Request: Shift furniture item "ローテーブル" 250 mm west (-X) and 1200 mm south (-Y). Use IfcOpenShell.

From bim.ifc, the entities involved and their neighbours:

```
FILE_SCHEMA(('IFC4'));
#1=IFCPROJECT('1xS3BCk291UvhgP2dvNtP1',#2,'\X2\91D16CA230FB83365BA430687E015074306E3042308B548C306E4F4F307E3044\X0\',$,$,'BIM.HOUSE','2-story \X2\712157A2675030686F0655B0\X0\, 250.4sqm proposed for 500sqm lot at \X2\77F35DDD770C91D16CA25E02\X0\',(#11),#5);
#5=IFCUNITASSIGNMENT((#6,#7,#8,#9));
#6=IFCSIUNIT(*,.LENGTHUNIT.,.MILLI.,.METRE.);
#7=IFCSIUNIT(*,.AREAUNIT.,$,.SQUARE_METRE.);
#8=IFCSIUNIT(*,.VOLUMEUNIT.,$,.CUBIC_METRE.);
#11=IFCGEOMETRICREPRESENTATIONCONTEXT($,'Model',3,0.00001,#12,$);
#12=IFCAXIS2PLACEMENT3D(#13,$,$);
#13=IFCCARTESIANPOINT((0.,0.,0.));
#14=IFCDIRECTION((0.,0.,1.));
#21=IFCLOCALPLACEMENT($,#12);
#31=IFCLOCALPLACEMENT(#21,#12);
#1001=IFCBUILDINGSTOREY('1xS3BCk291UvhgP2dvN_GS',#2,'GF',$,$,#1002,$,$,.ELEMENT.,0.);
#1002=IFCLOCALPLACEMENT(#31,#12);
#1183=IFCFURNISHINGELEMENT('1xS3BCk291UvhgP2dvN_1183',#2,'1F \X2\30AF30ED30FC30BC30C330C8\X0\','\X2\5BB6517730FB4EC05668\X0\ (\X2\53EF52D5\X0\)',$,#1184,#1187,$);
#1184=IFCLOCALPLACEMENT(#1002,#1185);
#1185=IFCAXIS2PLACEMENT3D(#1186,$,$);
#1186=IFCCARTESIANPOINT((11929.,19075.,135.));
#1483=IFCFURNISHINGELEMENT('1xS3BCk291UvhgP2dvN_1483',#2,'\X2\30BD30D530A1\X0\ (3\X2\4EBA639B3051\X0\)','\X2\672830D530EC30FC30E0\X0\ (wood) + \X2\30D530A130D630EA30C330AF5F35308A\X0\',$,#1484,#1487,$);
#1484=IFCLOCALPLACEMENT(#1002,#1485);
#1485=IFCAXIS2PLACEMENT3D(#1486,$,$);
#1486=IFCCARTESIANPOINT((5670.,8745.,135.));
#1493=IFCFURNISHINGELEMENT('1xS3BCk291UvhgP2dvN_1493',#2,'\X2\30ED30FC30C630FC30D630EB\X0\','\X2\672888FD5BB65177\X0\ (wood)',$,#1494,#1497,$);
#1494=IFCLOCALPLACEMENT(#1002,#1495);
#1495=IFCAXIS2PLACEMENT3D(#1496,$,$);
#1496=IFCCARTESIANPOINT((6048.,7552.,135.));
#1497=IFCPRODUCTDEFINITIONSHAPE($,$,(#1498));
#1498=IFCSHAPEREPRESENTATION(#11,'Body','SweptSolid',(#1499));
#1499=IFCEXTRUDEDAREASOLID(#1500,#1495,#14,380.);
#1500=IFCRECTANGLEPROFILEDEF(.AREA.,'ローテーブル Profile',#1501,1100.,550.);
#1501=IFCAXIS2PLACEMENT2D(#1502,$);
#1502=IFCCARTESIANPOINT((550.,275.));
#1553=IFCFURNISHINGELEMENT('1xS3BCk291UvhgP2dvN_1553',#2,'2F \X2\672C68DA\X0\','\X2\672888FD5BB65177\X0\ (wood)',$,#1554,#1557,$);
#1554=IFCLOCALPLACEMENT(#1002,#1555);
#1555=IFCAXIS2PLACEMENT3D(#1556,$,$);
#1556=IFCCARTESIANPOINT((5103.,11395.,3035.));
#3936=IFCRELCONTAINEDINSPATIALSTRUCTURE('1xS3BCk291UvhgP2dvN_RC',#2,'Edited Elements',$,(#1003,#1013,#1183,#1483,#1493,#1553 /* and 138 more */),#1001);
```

```python
import ifcopenshell
import ifcopenshell.api.geometry
import ifcopenshell.util.placement

model = ifcopenshell.open("bim.ifc")

item = model.by_id(1493)
matrix = ifcopenshell.util.placement.get_local_placement(item.ObjectPlacement)
matrix[0, 3] -= 250.0
matrix[1, 3] -= 1200.0
ifcopenshell.api.geometry.edit_object_placement(model, product=item, matrix=matrix, is_si=False)

print(ifcopenshell.util.placement.get_local_placement(item.ObjectPlacement).round(3) + 0.0)

model.write("bim_rev.ifc")
```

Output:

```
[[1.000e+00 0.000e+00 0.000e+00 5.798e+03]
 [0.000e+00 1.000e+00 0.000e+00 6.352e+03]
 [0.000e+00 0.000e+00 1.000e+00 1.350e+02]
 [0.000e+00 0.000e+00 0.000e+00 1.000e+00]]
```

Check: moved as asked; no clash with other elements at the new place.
